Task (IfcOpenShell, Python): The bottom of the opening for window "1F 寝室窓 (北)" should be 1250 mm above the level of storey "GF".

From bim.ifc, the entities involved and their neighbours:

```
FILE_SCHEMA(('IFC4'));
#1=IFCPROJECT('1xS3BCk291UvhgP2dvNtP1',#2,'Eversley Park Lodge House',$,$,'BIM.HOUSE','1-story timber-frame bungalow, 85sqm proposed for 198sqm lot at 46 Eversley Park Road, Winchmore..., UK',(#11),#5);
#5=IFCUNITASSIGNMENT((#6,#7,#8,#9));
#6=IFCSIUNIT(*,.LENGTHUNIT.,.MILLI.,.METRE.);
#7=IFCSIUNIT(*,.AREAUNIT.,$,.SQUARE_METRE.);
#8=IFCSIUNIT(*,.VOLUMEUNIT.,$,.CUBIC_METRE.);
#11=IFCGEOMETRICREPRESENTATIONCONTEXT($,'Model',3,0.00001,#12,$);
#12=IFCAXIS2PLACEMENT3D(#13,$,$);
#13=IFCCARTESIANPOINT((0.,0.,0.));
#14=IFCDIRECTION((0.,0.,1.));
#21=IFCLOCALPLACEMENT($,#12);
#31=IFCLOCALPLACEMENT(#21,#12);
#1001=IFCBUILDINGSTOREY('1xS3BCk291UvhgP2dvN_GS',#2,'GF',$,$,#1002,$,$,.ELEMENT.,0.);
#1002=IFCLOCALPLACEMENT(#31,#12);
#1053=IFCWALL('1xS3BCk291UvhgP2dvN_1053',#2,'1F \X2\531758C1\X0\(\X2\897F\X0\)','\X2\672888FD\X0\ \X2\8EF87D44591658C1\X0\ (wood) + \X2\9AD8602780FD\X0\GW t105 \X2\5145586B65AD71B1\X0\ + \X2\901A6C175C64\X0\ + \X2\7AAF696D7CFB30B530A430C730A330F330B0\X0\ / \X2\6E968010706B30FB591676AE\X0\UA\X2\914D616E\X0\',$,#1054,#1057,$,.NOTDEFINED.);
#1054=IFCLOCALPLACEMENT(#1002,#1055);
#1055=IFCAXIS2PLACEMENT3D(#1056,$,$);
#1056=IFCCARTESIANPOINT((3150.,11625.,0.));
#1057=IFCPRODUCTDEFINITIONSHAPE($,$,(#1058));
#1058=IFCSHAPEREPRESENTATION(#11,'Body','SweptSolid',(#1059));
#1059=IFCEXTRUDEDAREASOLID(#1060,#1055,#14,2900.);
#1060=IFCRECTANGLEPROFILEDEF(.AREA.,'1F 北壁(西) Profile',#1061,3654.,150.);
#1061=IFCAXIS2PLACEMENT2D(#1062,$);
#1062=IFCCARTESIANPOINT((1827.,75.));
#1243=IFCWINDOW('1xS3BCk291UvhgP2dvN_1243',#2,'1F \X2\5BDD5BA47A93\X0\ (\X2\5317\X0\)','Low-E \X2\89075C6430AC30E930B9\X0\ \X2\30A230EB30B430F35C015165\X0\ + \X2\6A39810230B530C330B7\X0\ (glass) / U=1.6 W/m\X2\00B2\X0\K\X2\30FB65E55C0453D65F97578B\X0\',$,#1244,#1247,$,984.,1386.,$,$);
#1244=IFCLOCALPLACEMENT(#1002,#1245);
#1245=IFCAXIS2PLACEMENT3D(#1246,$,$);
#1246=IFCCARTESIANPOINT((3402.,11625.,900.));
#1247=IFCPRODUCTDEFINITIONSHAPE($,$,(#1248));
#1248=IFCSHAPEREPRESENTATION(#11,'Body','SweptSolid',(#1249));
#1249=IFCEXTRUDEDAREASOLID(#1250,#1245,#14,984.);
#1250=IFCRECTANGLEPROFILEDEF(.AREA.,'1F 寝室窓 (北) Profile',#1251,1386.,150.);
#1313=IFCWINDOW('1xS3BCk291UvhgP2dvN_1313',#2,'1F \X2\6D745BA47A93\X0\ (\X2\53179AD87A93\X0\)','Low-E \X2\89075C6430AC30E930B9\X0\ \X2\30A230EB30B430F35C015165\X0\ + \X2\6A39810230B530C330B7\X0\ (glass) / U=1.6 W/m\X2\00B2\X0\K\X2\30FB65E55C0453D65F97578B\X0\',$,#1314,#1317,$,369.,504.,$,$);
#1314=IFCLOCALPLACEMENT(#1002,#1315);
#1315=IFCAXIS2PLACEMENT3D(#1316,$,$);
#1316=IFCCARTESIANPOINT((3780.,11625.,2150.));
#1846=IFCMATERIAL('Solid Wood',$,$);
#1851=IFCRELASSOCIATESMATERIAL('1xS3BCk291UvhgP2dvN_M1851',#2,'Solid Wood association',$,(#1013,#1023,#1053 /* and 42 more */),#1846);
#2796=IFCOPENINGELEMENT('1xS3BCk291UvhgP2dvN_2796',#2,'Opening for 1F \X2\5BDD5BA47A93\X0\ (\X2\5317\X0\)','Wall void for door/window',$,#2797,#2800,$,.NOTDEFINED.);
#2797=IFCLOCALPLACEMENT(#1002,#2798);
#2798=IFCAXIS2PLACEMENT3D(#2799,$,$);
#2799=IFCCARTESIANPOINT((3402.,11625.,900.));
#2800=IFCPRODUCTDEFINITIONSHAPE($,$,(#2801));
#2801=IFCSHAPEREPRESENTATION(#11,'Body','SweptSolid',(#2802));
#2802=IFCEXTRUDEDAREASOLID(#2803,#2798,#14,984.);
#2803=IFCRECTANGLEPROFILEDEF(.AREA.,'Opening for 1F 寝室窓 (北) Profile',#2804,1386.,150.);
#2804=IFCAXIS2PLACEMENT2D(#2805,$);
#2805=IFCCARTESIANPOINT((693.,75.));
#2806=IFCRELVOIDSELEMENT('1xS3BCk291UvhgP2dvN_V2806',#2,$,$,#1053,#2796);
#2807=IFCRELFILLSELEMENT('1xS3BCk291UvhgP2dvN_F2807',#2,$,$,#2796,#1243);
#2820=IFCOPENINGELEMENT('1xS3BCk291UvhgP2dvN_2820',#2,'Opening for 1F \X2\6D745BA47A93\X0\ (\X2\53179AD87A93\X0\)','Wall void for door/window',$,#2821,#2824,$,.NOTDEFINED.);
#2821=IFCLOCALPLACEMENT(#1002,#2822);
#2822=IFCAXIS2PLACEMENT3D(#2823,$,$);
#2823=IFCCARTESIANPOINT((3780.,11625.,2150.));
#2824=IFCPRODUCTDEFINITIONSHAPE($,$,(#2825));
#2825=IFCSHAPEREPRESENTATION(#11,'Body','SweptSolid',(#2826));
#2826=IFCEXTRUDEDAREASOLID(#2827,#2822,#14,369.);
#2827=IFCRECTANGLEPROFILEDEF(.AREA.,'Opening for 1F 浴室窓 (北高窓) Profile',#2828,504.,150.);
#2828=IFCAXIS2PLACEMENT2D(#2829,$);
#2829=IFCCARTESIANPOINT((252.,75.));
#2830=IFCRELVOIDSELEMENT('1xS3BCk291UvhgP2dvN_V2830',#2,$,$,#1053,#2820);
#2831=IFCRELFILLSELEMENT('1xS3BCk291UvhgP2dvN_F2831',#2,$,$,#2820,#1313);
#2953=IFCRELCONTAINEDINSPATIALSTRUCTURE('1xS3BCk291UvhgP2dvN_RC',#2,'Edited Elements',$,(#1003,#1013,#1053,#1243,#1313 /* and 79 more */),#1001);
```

```python
import numpy as np
import ifcopenshell
import ifcopenshell.api.geometry
import ifcopenshell.geom
import ifcopenshell.util.element
import ifcopenshell.util.placement
import ifcopenshell.util.shape
import ifcopenshell.util.unit

model = ifcopenshell.open("bim.ifc")
unit_scale = ifcopenshell.util.unit.calculate_unit_scale(model)

window = model.by_guid("1xS3BCk291UvhgP2dvN_1243")
opening = window.FillsVoids[0].RelatingOpeningElement
storey = ifcopenshell.util.element.get_container(window, ifc_class="IfcBuildingStorey")
level = ifcopenshell.util.placement.get_local_placement(storey.ObjectPlacement)[2, 3]

# The opening's origin need not be at the sill, so measure its lowest point.
shape = ifcopenshell.geom.create_shape(ifcopenshell.geom.settings(), opening)
bottom = ifcopenshell.util.shape.get_shape_bottom_elevation(shape, shape.geometry) / unit_scale
dz = level + 1.25 / unit_scale - bottom

shift = np.array([0.0, 0.0, dz])
# The window is not placed relative to its opening, so move both.
for product in (opening, window):
    matrix = ifcopenshell.util.placement.get_local_placement(product.ObjectPlacement)
    matrix[:3, 3] += shift
    ifcopenshell.api.geometry.edit_object_placement(model, product=product, matrix=matrix, is_si=False)

print(f"moved by {dz * unit_scale:+.3f} m")

model.write("bim_updated.ifc")
```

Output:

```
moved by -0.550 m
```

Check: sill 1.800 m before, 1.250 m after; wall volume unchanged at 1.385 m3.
